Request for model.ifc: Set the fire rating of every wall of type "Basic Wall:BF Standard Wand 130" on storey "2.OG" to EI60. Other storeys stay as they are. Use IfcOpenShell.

First a look at what the model holds.

```python
import ifcopenshell
import ifcopenshell.util.element

model = ifcopenshell.open("model.ifc")
print(model.schema)
storey = next(s for s in model.by_type("IfcBuildingStorey") if s.Name == "2.OG")
walls = [e for e in ifcopenshell.util.element.get_decomposition(storey) if e.is_a("IfcWall")]
seen = {}
for e in walls:
    element_type = ifcopenshell.util.element.get_type(e)
    key = (element_type.Name if element_type != e and element_type else None, ifcopenshell.util.element.get_pset(e, "Pset_WallCommon", "FireRating"))
    seen[key] = seen.get(key, 0) + 1
for (name, value), count in sorted(seen.items(), key=str):
    print(count, "x", name, "|", value)
```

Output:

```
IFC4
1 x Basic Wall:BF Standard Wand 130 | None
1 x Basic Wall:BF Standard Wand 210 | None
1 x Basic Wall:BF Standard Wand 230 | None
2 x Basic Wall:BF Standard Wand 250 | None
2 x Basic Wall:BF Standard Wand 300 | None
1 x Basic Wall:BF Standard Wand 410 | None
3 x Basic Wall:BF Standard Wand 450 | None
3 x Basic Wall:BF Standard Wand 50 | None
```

```python
import ifcopenshell
import ifcopenshell.api.pset
import ifcopenshell.util.element

model = ifcopenshell.open("model.ifc")

storey = next(s for s in model.by_type("IfcBuildingStorey") if s.Name == "2.OG")
walls = [e for e in ifcopenshell.util.element.get_decomposition(storey) if e.is_a("IfcWall")]

count = 0
for e in walls:
    element_type = ifcopenshell.util.element.get_type(e)
    if element_type in (None, e) or element_type.Name != "Basic Wall:BF Standard Wand 130":
        continue
    # add_pset returns the element's existing set when there is one.
    pset = ifcopenshell.api.pset.add_pset(model, product=e, name="Pset_WallCommon")
    ifcopenshell.api.pset.edit_pset(model, pset=pset, properties={"FireRating": "EI60"})
    count += 1

print(count, "walls updated")

model.write("model_v2.ifc")
```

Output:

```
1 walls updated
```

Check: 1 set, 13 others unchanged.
